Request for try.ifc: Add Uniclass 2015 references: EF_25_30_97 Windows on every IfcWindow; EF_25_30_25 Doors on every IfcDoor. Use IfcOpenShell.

First a look at what the model holds.

```python
import ifcopenshell

model = ifcopenshell.open("try.ifc")
print(model.schema)
print("classifications:", [c.Name for c in model.by_type("IfcClassification")])
for ifc_class in ("IfcDoor", "IfcRoof", "IfcStair", "IfcWall", "IfcWindow"):
    print(ifc_class, len(model.by_type(ifc_class)))
```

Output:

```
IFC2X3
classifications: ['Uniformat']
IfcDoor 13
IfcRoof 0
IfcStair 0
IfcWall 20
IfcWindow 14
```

```python
import ifcopenshell
import ifcopenshell.api.classification

model = ifcopenshell.open("try.ifc")

# IFC2X3 requires Source and Edition and has no link from the project to the system.
system = model.create_entity("IfcClassification", Source="NBS", Edition="2015", Name="Uniclass 2015")

codes = {
    "IfcWindow": ("EF_25_30_97", "Windows"),
    "IfcDoor": ("EF_25_30_25", "Doors"),
}
for ifc_class, (code, name) in codes.items():
    products = model.by_type(ifc_class)
    ifcopenshell.api.classification.add_reference(
        model, products=products, classification=system, identification=code, name=name
    )
    print(code, len(products))

model.write("try_edited.ifc")
```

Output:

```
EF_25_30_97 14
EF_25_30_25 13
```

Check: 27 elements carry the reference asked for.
